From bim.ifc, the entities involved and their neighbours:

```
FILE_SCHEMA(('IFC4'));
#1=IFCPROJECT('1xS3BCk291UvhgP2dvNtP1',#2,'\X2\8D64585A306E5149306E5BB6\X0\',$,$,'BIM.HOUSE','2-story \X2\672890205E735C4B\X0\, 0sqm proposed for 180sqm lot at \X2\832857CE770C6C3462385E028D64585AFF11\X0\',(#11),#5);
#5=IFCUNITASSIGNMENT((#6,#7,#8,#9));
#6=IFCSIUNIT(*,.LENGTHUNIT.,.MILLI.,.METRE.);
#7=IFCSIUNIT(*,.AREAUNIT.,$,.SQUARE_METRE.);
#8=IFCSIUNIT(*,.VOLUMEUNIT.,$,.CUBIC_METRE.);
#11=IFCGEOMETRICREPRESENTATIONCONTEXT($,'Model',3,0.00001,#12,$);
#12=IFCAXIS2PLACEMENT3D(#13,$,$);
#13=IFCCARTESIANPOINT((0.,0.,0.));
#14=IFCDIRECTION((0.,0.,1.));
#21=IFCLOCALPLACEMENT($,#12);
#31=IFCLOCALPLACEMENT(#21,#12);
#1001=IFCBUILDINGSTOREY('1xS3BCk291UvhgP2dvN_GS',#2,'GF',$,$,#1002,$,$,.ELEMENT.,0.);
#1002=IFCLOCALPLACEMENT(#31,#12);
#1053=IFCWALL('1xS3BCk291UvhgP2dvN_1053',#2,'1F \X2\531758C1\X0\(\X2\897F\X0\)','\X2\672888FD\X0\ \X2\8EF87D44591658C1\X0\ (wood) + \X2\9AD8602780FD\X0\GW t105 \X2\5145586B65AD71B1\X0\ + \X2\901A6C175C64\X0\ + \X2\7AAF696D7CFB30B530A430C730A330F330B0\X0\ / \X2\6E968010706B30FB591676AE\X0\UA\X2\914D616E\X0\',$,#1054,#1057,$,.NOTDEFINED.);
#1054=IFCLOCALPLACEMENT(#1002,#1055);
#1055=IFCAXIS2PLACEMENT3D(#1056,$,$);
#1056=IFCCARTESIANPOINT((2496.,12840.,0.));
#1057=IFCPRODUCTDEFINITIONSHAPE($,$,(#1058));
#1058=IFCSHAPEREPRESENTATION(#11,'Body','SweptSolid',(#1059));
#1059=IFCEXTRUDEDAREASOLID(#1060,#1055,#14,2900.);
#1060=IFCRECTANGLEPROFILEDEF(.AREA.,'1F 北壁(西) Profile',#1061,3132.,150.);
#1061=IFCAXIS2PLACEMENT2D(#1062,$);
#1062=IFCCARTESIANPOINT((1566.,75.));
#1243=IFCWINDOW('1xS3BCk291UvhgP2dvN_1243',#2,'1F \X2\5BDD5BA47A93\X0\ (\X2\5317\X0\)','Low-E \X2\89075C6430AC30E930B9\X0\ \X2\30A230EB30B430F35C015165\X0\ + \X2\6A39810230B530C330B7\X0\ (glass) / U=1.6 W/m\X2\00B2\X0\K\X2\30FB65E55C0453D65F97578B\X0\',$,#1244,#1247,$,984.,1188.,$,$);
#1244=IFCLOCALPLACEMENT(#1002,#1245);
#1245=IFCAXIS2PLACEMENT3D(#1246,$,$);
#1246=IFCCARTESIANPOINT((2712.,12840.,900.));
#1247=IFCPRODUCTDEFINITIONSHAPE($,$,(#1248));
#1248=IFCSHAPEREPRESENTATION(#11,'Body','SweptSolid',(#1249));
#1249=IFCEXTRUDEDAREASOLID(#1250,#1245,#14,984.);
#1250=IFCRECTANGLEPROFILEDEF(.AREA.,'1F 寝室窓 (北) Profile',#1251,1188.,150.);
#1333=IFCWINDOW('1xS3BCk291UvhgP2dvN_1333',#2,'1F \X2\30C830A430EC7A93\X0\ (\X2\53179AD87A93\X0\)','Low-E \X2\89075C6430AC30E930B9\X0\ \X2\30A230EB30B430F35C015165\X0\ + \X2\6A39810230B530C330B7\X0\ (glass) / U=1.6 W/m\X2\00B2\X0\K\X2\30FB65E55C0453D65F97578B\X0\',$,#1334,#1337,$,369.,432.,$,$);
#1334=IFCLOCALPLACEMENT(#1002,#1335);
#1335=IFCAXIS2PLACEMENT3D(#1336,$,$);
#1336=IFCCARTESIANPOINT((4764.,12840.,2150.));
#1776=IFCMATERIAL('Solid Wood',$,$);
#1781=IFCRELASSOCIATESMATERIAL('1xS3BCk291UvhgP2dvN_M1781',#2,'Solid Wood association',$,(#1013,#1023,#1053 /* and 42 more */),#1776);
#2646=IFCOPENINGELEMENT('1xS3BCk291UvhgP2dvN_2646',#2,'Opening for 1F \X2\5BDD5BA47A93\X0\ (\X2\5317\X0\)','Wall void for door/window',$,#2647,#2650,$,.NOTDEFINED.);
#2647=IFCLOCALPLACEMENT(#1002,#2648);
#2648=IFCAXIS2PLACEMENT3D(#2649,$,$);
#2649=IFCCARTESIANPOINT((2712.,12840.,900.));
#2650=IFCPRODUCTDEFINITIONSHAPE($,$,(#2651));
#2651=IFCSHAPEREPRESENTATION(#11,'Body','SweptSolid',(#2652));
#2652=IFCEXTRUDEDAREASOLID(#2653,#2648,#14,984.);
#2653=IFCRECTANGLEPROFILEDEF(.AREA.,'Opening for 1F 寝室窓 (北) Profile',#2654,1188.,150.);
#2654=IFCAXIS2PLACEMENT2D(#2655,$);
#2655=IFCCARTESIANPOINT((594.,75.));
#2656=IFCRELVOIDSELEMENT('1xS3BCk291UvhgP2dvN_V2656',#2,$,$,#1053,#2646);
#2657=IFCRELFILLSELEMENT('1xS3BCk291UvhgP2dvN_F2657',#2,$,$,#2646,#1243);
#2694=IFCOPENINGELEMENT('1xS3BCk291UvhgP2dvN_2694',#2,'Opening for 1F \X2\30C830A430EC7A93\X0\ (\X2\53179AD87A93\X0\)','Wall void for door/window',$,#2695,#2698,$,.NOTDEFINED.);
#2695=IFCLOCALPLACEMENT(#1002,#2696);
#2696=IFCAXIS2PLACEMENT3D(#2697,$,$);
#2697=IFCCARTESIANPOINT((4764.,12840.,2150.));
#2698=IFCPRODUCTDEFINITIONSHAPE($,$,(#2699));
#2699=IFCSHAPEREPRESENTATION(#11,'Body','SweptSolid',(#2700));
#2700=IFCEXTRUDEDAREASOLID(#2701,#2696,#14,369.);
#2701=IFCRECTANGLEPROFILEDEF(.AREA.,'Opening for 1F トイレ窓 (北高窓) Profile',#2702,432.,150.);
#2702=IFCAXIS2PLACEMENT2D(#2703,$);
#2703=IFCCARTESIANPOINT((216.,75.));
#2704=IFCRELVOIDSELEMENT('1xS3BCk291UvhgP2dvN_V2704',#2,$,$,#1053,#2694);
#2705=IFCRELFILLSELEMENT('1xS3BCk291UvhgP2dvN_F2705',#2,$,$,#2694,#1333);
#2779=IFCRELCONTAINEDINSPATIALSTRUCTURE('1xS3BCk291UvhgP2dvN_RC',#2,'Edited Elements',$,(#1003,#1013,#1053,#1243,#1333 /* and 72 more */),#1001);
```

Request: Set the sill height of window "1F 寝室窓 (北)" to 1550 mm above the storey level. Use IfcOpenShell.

```python
import numpy as np
import ifcopenshell
import ifcopenshell.api.geometry
import ifcopenshell.geom
import ifcopenshell.util.element
import ifcopenshell.util.placement
import ifcopenshell.util.shape
import ifcopenshell.util.unit

model = ifcopenshell.open("bim.ifc")
unit_scale = ifcopenshell.util.unit.calculate_unit_scale(model)

window = model.by_id(1243)
opening = window.FillsVoids[0].RelatingOpeningElement
storey = ifcopenshell.util.element.get_container(window, ifc_class="IfcBuildingStorey")
level = ifcopenshell.util.placement.get_local_placement(storey.ObjectPlacement)[2, 3]

# The opening's origin need not be at the sill, so measure its lowest point.
shape = ifcopenshell.geom.create_shape(ifcopenshell.geom.settings(), opening)
bottom = ifcopenshell.util.shape.get_shape_bottom_elevation(shape, shape.geometry) / unit_scale
dz = level + 1.55 / unit_scale - bottom

shift = np.array([0.0, 0.0, dz])
# The window is not placed relative to its opening, so move both.
for product in (opening, window):
    matrix = ifcopenshell.util.placement.get_local_placement(product.ObjectPlacement)
    matrix[:3, 3] += shift
    ifcopenshell.api.geometry.edit_object_placement(model, product=product, matrix=matrix, is_si=False)

print(f"moved by {dz * unit_scale:+.3f} m")

model.write("bim_v2.ifc")
```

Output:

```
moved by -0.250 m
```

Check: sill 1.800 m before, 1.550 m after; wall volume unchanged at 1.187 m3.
